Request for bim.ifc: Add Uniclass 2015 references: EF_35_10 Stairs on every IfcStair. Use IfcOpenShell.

First a look at what the model holds.

```python
import ifcopenshell

model = ifcopenshell.open("bim.ifc")
print(model.schema)
print("classifications:", [c.Name for c in model.by_type("IfcClassification")])
for ifc_class in ("IfcDoor", "IfcRoof", "IfcStair", "IfcWall", "IfcWindow"):
    print(ifc_class, len(model.by_type(ifc_class)))
```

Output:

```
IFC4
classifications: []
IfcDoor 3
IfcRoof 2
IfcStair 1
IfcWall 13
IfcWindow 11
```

```python
import ifcopenshell
import ifcopenshell.api.classification

model = ifcopenshell.open("bim.ifc")

system = ifcopenshell.api.classification.add_classification(model, classification="Uniclass 2015")

codes = {
    "IfcStair": ("EF_35_10", "Stairs"),
}
for ifc_class, (code, name) in codes.items():
    products = model.by_type(ifc_class)
    ifcopenshell.api.classification.add_reference(
        model, products=products, classification=system, identification=code, name=name
    )
    print(code, len(products))

model.write("bim-out.ifc")
```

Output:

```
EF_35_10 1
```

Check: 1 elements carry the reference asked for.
